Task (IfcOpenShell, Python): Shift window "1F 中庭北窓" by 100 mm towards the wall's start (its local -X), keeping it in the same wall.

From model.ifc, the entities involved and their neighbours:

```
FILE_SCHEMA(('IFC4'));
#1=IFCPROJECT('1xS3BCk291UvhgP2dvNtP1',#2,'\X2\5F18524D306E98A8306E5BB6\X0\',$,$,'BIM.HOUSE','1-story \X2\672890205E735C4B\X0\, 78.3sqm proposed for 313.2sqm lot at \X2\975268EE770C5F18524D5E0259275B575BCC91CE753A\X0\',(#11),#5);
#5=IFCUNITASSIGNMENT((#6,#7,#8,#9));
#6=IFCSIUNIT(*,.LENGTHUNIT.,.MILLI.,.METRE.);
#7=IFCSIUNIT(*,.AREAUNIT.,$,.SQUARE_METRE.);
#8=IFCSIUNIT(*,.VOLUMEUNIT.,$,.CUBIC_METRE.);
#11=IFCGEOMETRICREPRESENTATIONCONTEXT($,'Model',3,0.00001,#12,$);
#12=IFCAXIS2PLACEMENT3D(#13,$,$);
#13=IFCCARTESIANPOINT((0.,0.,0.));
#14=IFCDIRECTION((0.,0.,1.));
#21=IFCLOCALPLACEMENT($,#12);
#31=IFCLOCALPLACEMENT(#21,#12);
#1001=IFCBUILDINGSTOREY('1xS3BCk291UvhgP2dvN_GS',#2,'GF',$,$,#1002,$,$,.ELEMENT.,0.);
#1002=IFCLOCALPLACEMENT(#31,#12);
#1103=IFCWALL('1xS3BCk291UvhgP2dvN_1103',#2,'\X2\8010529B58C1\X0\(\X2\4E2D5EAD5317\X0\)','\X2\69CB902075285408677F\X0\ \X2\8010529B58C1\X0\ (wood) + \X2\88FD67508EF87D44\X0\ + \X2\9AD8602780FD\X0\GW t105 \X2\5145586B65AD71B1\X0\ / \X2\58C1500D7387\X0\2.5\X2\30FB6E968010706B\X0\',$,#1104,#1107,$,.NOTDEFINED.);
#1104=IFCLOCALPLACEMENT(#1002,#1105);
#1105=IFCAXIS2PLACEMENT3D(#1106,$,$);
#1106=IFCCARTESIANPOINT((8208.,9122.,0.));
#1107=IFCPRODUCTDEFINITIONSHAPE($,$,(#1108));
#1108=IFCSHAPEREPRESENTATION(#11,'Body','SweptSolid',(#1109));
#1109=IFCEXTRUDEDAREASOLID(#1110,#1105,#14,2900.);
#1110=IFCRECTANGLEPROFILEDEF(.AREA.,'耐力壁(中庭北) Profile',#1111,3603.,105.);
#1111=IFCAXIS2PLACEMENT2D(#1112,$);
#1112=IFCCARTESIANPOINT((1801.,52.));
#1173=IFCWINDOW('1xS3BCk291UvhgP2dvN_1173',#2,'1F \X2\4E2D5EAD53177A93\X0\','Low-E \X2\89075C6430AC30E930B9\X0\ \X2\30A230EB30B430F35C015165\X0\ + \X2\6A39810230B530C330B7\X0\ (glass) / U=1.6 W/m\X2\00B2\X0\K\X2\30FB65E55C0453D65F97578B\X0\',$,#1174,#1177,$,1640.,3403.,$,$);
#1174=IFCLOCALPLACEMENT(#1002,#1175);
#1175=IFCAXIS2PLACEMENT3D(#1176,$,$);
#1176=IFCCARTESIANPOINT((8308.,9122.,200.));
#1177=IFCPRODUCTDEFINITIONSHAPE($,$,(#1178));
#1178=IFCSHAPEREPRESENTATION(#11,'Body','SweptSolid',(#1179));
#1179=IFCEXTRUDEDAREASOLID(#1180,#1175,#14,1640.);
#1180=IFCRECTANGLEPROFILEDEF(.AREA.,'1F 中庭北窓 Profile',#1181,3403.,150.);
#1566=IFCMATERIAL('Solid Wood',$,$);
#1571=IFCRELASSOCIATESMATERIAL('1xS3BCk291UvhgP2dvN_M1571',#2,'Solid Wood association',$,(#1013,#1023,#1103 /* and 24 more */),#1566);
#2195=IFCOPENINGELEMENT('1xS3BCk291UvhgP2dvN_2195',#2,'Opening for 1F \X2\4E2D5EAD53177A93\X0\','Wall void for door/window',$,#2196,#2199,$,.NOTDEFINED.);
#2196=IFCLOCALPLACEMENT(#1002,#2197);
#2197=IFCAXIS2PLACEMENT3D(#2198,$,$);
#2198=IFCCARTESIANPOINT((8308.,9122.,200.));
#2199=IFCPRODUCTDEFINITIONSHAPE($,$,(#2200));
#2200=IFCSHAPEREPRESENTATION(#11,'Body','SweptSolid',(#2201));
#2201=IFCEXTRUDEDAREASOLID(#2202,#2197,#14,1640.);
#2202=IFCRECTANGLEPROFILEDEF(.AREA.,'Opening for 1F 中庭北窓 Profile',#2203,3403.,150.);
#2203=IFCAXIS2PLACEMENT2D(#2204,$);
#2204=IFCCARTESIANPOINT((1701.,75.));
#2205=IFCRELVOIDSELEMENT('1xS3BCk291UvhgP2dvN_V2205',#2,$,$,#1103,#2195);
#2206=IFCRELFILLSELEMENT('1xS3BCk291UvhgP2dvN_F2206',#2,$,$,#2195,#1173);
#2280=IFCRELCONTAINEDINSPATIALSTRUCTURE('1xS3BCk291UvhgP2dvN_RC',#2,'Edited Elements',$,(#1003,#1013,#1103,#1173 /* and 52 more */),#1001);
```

```python
import ifcopenshell
import ifcopenshell.api.geometry
import ifcopenshell.util.placement

model = ifcopenshell.open("model.ifc")

window = model.by_guid("1xS3BCk291UvhgP2dvN_1173")
opening = window.FillsVoids[0].RelatingOpeningElement
wall = opening.VoidsElements[0].RelatingBuildingElement

wall_matrix = ifcopenshell.util.placement.get_local_placement(wall.ObjectPlacement)
shift = wall_matrix[:3, 0] * -100.0
before = ifcopenshell.util.placement.get_local_placement(window.ObjectPlacement)[:3, 3].copy()

# The window is not placed relative to its opening, so move both.
for product in (opening, window):
    matrix = ifcopenshell.util.placement.get_local_placement(product.ObjectPlacement)
    matrix[:3, 3] += shift
    ifcopenshell.api.geometry.edit_object_placement(model, product=product, matrix=matrix, is_si=False)

after = ifcopenshell.util.placement.get_local_placement(window.ObjectPlacement)[:3, 3]
print("window moved by", (after - before).round(3) + 0.0)

model.write("model-out.ifc")
```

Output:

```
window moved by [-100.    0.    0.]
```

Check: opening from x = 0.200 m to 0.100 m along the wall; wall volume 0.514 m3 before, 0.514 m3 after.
